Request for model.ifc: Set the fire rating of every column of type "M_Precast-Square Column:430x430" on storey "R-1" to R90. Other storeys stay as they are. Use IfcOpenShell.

First a look at what the model holds.

```python
import ifcopenshell
import ifcopenshell.util.element

model = ifcopenshell.open("model.ifc")
print(model.schema)
storey = next(s for s in model.by_type("IfcBuildingStorey") if s.Name == "R-1")
columns = [e for e in ifcopenshell.util.element.get_decomposition(storey) if e.is_a("IfcColumn")]
seen = {}
for e in columns:
    element_type = ifcopenshell.util.element.get_type(e)
    key = (element_type.Name if element_type != e and element_type else None, ifcopenshell.util.element.get_pset(e, "Pset_ColumnCommon", "FireRating"))
    seen[key] = seen.get(key, 0) + 1
for (name, value), count in sorted(seen.items(), key=str):
    print(count, "x", name, "|", value)
```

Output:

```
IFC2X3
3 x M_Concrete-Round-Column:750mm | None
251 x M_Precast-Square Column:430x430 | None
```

```python
import ifcopenshell
import ifcopenshell.api.pset
import ifcopenshell.util.element

model = ifcopenshell.open("model.ifc")

storey = next(s for s in model.by_type("IfcBuildingStorey") if s.Name == "R-1")
columns = [e for e in ifcopenshell.util.element.get_decomposition(storey) if e.is_a("IfcColumn")]

count = 0
for e in columns:
    element_type = ifcopenshell.util.element.get_type(e)
    if element_type in (None, e) or element_type.Name != "M_Precast-Square Column:430x430":
        continue
    # add_pset returns the element's existing set when there is one.
    pset = ifcopenshell.api.pset.add_pset(model, product=e, name="Pset_ColumnCommon")
    ifcopenshell.api.pset.edit_pset(model, pset=pset, properties={"FireRating": "R90"})
    count += 1

print(count, "columns updated")

model.write("model_updated.ifc")
```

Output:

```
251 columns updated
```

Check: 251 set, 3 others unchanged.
